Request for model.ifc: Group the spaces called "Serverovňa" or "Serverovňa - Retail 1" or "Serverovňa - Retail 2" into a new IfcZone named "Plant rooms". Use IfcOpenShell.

First a look at what the model holds.

```python
import ifcopenshell

model = ifcopenshell.open("model.ifc")
print(model.schema)
seen = {}
for space in model.by_type("IfcSpace"):
    seen[space.LongName] = seen.get(space.LongName, 0) + 1
for name, count in sorted(seen.items(), key=str):
    print(count, "x", name)
print("zones:", [z.Name for z in model.by_type("IfcZone")][:20])
```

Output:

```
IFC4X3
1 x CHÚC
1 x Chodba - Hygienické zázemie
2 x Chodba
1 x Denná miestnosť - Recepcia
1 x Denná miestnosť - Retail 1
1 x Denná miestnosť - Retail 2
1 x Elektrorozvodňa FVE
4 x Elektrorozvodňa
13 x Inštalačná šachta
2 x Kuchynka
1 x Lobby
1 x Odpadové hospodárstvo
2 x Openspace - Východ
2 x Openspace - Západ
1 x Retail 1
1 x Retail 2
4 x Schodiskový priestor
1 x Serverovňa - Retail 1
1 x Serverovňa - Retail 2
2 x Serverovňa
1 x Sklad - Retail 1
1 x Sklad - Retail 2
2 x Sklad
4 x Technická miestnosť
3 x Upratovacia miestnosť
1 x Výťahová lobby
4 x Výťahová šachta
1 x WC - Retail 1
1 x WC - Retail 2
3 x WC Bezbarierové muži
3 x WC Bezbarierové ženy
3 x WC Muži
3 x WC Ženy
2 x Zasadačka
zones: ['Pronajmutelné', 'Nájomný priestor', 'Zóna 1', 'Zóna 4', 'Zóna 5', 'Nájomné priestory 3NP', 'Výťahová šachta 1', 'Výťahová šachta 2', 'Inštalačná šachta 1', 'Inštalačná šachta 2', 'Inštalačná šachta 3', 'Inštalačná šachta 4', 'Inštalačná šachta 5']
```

```python
import ifcopenshell
import ifcopenshell.api.group
import ifcopenshell.api.root

model = ifcopenshell.open("model.ifc")

names = {"Serverovňa", "Serverovňa - Retail 1", "Serverovňa - Retail 2"}
spaces = [s for s in model.by_type("IfcSpace") if s.LongName in names]

zone = ifcopenshell.api.root.create_entity(model, ifc_class="IfcZone", name="Plant rooms")
ifcopenshell.api.group.assign_group(model, products=spaces, group=zone)
print(len(spaces), "spaces in", zone.Name)

model.write("model_v2.ifc")
```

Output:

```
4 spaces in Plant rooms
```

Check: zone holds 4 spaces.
